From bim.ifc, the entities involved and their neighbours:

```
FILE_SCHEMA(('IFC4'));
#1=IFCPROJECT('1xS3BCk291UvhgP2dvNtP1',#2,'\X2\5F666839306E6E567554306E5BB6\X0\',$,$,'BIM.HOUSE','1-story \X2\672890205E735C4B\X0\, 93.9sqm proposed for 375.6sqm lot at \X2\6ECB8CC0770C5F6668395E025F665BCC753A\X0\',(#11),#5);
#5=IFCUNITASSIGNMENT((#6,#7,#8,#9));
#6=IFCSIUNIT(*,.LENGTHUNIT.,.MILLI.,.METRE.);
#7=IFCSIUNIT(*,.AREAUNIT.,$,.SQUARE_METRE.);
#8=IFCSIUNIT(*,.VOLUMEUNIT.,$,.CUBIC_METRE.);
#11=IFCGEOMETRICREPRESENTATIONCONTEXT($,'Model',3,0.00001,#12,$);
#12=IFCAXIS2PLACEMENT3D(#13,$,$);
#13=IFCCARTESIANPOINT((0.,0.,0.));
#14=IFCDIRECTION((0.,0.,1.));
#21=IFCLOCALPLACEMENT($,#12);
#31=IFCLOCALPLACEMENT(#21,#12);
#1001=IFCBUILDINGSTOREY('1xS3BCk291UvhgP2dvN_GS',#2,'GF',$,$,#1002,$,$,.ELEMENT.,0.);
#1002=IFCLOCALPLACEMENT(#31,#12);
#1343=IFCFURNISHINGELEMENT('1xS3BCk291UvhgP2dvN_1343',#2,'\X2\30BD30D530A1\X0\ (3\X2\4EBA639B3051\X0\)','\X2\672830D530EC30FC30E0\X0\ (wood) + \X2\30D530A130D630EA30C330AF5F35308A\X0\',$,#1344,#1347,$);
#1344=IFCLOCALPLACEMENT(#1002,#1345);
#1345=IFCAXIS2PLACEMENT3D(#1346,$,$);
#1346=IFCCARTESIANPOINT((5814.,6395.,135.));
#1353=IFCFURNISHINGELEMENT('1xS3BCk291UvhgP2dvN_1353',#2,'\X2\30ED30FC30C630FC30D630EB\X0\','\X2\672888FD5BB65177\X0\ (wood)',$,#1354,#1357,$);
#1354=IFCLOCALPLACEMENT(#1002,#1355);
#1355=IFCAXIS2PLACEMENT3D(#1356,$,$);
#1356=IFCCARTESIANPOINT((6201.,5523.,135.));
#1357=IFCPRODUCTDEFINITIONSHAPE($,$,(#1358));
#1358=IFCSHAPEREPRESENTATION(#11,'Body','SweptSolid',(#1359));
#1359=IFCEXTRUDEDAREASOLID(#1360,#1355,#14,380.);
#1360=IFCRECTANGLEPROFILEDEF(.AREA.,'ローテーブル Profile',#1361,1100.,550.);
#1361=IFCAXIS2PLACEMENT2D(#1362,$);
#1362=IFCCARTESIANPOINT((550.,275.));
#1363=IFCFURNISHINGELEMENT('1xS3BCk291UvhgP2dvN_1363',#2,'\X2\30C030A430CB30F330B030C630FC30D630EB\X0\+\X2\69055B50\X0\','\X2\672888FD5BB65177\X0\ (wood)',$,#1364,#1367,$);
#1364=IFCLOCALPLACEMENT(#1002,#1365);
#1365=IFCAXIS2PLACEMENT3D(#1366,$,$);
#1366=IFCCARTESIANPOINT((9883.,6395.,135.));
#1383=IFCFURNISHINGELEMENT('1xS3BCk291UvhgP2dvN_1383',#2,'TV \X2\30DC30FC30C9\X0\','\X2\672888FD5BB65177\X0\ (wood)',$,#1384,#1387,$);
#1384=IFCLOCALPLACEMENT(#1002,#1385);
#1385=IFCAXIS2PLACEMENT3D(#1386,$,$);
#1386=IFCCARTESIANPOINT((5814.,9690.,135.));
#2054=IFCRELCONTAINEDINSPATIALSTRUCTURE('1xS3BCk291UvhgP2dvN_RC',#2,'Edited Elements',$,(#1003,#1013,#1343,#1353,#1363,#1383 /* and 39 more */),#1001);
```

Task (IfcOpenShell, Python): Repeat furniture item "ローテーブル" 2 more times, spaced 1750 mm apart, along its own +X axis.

```python
import ifcopenshell
import ifcopenshell.api.geometry
import ifcopenshell.api.root
import ifcopenshell.util.element
import ifcopenshell.util.placement
import ifcopenshell.util.unit

model = ifcopenshell.open("bim.ifc")
unit_scale = ifcopenshell.util.unit.calculate_unit_scale(model)


def reuse_history(source, copy):
    """copy_class also copies each property set's owner history, people and application; keep the originals."""
    for rel in copy.IsDefinedBy:
        if rel.is_a("IfcRelDefinesByProperties") and (history := rel.RelatingPropertyDefinition.OwnerHistory):
            rel.RelatingPropertyDefinition.OwnerHistory = source.OwnerHistory
            ifcopenshell.util.element.remove_deep2(model, history)


source = model.by_id(1353)
base = ifcopenshell.util.placement.get_local_placement(source.ObjectPlacement)
step = base[:3, 0] * 1.75 / unit_scale

for i in range(1, 3):
    copy = ifcopenshell.api.root.copy_class(model, product=source)
    copy.Representation = ifcopenshell.util.element.copy_deep(
        model, source.Representation, exclude=["IfcGeometricRepresentationContext", "IfcRepresentationMap"]
    )
    reuse_history(source, copy)
    matrix = base.copy()
    matrix[:3, 3] += i * step
    print("added at", matrix[:3, 3].round(3) + 0.0)
    ifcopenshell.api.geometry.edit_object_placement(model, product=copy, matrix=matrix, is_si=False)

model.write("bim_updated.ifc")
```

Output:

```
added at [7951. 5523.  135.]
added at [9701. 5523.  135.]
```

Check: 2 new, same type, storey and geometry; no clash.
